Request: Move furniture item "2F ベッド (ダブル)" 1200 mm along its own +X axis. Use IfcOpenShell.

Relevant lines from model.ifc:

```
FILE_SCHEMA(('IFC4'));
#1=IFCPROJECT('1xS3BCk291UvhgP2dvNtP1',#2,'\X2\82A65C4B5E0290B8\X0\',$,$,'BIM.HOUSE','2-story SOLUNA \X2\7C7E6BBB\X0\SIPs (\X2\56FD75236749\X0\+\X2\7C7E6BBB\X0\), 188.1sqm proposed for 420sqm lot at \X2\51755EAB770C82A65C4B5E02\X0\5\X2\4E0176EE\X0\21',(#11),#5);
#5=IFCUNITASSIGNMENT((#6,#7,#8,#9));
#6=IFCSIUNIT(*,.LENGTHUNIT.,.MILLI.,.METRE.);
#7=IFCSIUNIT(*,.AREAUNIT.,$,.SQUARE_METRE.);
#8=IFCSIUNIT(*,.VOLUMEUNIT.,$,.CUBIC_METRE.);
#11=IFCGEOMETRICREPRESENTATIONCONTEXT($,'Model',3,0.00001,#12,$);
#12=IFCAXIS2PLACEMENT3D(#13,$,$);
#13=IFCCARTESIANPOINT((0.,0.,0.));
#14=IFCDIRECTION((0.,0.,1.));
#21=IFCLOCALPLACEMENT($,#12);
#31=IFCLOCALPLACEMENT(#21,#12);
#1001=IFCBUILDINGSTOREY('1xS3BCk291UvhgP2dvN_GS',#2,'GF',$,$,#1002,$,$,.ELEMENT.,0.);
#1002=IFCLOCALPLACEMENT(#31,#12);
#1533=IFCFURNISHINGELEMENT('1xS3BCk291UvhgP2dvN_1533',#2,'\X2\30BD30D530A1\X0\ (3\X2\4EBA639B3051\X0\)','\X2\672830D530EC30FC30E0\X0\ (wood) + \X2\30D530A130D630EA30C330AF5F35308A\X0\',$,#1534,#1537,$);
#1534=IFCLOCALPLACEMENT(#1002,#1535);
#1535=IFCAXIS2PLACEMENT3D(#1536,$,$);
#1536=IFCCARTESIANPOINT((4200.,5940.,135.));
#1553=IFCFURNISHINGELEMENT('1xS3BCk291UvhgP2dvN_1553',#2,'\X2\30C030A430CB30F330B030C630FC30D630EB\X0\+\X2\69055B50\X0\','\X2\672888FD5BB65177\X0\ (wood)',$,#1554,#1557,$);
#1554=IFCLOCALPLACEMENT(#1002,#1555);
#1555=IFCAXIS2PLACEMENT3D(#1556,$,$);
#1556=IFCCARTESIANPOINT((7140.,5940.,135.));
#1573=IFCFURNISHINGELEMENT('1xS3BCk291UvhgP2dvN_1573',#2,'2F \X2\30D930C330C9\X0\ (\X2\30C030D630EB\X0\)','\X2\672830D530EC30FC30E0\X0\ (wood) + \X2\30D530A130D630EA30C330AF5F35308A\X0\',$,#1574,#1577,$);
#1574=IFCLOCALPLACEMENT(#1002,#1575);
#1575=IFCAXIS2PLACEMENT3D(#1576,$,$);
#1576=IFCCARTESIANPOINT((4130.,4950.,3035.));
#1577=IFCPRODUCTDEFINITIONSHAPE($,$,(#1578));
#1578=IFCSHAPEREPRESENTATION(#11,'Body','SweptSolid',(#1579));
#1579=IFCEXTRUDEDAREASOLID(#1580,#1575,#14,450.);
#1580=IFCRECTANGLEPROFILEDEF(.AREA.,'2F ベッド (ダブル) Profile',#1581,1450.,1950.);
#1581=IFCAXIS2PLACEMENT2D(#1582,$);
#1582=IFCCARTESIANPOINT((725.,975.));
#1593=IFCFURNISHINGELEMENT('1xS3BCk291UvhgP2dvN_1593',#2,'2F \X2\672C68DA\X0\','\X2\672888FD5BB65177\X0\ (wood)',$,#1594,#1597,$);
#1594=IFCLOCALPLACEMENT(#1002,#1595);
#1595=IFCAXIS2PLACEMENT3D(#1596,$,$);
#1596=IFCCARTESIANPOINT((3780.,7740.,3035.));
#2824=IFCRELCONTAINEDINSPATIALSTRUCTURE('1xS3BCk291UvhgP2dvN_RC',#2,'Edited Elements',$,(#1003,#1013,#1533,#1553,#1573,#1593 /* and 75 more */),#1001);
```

```python
import ifcopenshell
import ifcopenshell.api.geometry
import ifcopenshell.util.placement

model = ifcopenshell.open("model.ifc")

item = model.by_guid("1xS3BCk291UvhgP2dvN_1573")
matrix = ifcopenshell.util.placement.get_local_placement(item.ObjectPlacement)
matrix[:3, 3] += matrix[:3, 0] * 1200.0
ifcopenshell.api.geometry.edit_object_placement(model, product=item, matrix=matrix, is_si=False)

print(ifcopenshell.util.placement.get_local_placement(item.ObjectPlacement).round(3) + 0.0)

model.write("model_v2.ifc")
```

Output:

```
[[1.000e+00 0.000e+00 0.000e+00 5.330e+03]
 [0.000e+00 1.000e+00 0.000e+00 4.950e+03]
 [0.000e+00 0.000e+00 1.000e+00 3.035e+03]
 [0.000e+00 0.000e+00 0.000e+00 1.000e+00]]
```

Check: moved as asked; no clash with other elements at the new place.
